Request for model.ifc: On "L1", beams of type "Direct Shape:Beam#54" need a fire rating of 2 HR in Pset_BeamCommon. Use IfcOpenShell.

First a look at what the model holds.

```python
import ifcopenshell
import ifcopenshell.util.element

model = ifcopenshell.open("model.ifc")
print(model.schema)
storey = next(s for s in model.by_type("IfcBuildingStorey") if s.Name == "L1")
beams = [e for e in ifcopenshell.util.element.get_decomposition(storey) if e.is_a("IfcBeam")]
seen = {}
for e in beams:
    element_type = ifcopenshell.util.element.get_type(e)
    key = (element_type.Name if element_type != e and element_type else None, ifcopenshell.util.element.get_pset(e, "Pset_BeamCommon", "FireRating"))
    seen[key] = seen.get(key, 0) + 1
for (name, value), count in sorted(seen.items(), key=str):
    print(count, "x", name, "|", value)
```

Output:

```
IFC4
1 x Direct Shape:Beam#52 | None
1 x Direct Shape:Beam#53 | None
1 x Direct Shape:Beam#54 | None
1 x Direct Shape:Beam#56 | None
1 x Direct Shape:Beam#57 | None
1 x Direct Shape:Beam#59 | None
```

```python
import ifcopenshell
import ifcopenshell.api.pset
import ifcopenshell.util.element

model = ifcopenshell.open("model.ifc")

storey = next(s for s in model.by_type("IfcBuildingStorey") if s.Name == "L1")
beams = [e for e in ifcopenshell.util.element.get_decomposition(storey) if e.is_a("IfcBeam")]

count = 0
for e in beams:
    element_type = ifcopenshell.util.element.get_type(e)
    if element_type in (None, e) or element_type.Name != "Direct Shape:Beam#54":
        continue
    # add_pset returns the element's existing set when there is one.
    pset = ifcopenshell.api.pset.add_pset(model, product=e, name="Pset_BeamCommon")
    ifcopenshell.api.pset.edit_pset(model, pset=pset, properties={"FireRating": "2 HR"})
    count += 1

print(count, "beams updated")

model.write("model_v2.ifc")
```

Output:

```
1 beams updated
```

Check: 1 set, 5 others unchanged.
